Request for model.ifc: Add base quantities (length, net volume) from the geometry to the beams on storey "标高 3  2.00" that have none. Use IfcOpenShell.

First a look at what the model holds.

```python
import ifcopenshell
import ifcopenshell.util.element
import ifcopenshell.util.unit

model = ifcopenshell.open("model.ifc")
print(model.schema)
for unit_type in ("LENGTHUNIT", "AREAUNIT", "VOLUMEUNIT"):
    print(unit_type, ifcopenshell.util.unit.calculate_unit_scale(model, unit_type))
storey = next(s for s in model.by_type("IfcBuildingStorey") if s.Name == "标高 3  2.00")
beams = [e for e in ifcopenshell.util.element.get_decomposition(storey) if e.is_a("IfcBeam")]
for e in sorted(beams, key=lambda e: e.id()):
    print(e.id(), e.is_a(), e.Name, list(ifcopenshell.util.element.get_psets(e, qtos_only=True)), sep=" | ")
```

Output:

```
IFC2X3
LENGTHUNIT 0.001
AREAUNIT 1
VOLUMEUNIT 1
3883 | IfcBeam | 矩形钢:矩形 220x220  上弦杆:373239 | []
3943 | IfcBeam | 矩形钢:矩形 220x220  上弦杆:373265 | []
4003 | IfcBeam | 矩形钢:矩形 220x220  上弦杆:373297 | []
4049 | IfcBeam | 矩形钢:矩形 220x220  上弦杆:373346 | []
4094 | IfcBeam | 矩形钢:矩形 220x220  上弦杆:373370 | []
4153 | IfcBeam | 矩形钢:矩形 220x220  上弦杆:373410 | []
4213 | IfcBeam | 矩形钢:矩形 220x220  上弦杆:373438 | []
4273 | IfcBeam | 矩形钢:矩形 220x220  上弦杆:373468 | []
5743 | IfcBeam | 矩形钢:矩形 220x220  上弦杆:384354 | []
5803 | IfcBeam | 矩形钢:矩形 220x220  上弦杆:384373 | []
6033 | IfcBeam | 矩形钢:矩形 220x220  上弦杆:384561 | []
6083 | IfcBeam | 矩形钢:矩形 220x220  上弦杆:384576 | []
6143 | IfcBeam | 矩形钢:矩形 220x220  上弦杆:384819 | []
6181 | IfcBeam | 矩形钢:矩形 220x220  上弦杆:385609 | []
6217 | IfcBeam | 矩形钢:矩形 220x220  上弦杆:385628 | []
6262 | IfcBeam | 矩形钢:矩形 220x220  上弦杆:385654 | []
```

```python
import ifcopenshell
import ifcopenshell.api.pset
import ifcopenshell.geom
import ifcopenshell.util.element
import ifcopenshell.util.shape
import ifcopenshell.util.unit

model = ifcopenshell.open("model.ifc")
unit_scale = ifcopenshell.util.unit.calculate_unit_scale(model)
volume_scale = ifcopenshell.util.unit.calculate_unit_scale(model, "VOLUMEUNIT")
settings = ifcopenshell.geom.settings()

storey = next(s for s in model.by_type("IfcBuildingStorey") if s.Name == "标高 3  2.00")
beams = [e for e in ifcopenshell.util.element.get_decomposition(storey) if e.is_a("IfcBeam")]

for e in sorted(beams, key=lambda e: e.id()):
    if ifcopenshell.util.element.get_psets(e, qtos_only=True, should_inherit=False):
        continue
    # Geometry comes back in metres, in the element's own axes.
    shape = ifcopenshell.geom.create_shape(settings, e)
    values = {
        "Length": ifcopenshell.util.shape.get_max_xyz(shape.geometry) / unit_scale,
        "NetVolume": ifcopenshell.util.shape.get_volume(shape.geometry) / volume_scale,
    }
    qto = ifcopenshell.api.pset.add_qto(model, product=e, name="BaseQuantities")
    ifcopenshell.api.pset.edit_qto(model, qto=qto, properties=values)
    print(e.id(), {k: round(v, 3) for k, v in values.items()})

model.write("model_edited.ifc")
```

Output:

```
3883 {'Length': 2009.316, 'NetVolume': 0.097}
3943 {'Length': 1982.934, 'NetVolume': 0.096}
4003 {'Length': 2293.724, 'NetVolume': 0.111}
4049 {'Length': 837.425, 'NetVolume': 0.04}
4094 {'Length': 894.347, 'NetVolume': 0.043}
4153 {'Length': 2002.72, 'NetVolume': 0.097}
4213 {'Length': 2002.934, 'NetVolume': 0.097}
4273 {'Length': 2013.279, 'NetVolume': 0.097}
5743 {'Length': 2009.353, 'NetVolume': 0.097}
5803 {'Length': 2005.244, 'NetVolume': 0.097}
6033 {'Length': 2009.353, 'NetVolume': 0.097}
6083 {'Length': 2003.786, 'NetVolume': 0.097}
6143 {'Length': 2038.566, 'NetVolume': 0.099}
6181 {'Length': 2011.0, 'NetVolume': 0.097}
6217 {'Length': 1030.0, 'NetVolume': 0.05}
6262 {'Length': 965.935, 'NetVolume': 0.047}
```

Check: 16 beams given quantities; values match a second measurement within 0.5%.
